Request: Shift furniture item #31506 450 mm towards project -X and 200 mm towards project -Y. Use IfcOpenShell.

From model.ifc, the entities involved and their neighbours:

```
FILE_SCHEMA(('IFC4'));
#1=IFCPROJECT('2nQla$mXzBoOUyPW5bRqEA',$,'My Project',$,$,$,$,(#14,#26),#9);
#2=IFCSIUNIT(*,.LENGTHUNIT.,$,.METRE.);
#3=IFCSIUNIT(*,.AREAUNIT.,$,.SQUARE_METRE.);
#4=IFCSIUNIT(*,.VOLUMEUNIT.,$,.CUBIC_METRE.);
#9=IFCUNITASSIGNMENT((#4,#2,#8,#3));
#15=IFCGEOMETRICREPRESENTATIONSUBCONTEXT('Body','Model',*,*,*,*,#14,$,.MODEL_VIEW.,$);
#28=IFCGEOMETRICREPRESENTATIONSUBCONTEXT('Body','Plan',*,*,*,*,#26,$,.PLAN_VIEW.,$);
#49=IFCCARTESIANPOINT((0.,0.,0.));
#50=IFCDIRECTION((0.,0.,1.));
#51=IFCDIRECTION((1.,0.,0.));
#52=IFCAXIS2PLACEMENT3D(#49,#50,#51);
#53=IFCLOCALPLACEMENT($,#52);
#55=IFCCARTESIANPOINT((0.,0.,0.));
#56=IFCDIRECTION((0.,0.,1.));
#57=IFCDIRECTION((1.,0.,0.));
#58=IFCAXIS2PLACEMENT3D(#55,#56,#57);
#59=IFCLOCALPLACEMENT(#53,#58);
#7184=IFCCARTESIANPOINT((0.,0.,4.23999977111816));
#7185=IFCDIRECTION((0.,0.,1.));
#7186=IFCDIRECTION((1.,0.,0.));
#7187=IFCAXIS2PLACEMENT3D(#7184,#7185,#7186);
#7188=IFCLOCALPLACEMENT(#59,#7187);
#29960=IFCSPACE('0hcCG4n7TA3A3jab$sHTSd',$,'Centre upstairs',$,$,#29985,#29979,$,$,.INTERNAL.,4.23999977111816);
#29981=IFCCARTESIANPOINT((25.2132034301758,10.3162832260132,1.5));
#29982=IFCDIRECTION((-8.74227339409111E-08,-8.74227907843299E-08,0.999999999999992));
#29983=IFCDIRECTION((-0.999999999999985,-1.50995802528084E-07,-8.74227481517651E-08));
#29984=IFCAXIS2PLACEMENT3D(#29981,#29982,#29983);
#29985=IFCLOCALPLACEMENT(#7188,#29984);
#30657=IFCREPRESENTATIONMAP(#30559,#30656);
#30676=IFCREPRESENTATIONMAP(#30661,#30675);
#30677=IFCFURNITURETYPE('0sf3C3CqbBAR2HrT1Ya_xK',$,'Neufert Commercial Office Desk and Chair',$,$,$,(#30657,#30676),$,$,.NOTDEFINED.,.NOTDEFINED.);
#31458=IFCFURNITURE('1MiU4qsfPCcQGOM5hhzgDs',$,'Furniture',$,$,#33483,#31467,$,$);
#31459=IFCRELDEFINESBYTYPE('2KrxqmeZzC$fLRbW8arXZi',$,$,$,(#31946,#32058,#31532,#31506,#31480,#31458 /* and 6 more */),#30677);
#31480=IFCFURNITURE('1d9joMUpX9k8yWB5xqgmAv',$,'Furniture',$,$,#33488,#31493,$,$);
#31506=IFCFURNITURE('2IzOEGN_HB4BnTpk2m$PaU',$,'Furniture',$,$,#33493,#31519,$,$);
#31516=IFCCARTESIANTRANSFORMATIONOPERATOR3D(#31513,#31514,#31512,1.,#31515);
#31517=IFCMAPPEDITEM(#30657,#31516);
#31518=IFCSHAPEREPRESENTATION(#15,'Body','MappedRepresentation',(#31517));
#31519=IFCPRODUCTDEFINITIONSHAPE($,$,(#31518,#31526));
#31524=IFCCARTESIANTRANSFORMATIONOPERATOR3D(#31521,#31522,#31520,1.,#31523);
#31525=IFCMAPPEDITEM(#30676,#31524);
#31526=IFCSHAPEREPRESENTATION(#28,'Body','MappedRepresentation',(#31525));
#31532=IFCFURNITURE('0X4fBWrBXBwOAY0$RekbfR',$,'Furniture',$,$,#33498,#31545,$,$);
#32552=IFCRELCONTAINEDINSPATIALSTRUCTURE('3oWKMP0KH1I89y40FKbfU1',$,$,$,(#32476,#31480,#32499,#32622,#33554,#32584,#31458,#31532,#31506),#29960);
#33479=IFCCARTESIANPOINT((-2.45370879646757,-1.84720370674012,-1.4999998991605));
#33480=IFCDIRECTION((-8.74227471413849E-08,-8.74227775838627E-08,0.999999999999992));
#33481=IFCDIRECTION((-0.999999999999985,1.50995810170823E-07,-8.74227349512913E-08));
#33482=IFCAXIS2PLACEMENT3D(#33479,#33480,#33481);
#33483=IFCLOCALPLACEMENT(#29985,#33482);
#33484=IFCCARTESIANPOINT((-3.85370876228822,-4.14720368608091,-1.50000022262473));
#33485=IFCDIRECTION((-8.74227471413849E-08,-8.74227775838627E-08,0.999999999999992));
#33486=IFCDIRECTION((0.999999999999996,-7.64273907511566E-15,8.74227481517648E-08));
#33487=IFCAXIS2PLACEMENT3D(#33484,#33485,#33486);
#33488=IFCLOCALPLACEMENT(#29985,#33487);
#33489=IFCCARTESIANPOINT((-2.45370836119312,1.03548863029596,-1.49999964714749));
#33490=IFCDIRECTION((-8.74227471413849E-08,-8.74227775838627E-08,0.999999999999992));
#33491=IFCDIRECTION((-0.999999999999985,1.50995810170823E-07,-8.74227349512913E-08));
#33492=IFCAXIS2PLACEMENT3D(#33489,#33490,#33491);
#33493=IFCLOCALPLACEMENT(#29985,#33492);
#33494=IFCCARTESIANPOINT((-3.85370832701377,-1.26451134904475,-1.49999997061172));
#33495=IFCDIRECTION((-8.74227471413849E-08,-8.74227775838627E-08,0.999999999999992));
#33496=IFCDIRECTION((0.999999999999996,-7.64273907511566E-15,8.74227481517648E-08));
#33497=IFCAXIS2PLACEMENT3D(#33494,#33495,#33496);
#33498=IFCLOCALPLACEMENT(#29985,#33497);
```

```python
import ifcopenshell
import ifcopenshell.api.geometry
import ifcopenshell.util.placement
import ifcopenshell.util.unit

model = ifcopenshell.open("model.ifc")
unit_scale = ifcopenshell.util.unit.calculate_unit_scale(model)

item = model.by_id(31506)
matrix = ifcopenshell.util.placement.get_local_placement(item.ObjectPlacement)
matrix[0, 3] -= 0.45 / unit_scale
matrix[1, 3] -= 0.2 / unit_scale
ifcopenshell.api.geometry.edit_object_placement(model, product=item, matrix=matrix, is_si=False)

print(ifcopenshell.util.placement.get_local_placement(item.ObjectPlacement).round(3) + 0.0)

model.write("model_v2.ifc")
```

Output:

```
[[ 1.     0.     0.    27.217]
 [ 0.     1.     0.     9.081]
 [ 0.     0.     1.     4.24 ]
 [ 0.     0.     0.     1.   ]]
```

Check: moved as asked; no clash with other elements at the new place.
